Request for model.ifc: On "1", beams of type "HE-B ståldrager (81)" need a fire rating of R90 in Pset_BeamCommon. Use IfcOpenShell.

First a look at what the model holds.

```python
import ifcopenshell
import ifcopenshell.util.element

model = ifcopenshell.open("model.ifc")
print(model.schema)
storey = next(s for s in model.by_type("IfcBuildingStorey") if s.Name == "1")
beams = [e for e in ifcopenshell.util.element.get_decomposition(storey) if e.is_a("IfcBeam")]
seen = {}
for e in beams:
    element_type = ifcopenshell.util.element.get_type(e)
    key = (element_type.Name if element_type != e and element_type else None, ifcopenshell.util.element.get_pset(e, "Pset_BeamCommon", "FireRating"))
    seen[key] = seen.get(key, 0) + 1
for (name, value), count in sorted(seen.items(), key=str):
    print(count, "x", name, "|", value)
```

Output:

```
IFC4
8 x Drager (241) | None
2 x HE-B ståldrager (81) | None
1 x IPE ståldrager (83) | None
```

```python
import ifcopenshell
import ifcopenshell.api.pset
import ifcopenshell.util.element

model = ifcopenshell.open("model.ifc")

storey = next(s for s in model.by_type("IfcBuildingStorey") if s.Name == "1")
beams = [e for e in ifcopenshell.util.element.get_decomposition(storey) if e.is_a("IfcBeam")]

count = 0
for e in beams:
    element_type = ifcopenshell.util.element.get_type(e)
    if element_type in (None, e) or element_type.Name != "HE-B ståldrager (81)":
        continue
    # add_pset returns the element's existing set when there is one.
    pset = ifcopenshell.api.pset.add_pset(model, product=e, name="Pset_BeamCommon")
    ifcopenshell.api.pset.edit_pset(model, pset=pset, properties={"FireRating": "R90"})
    count += 1

print(count, "beams updated")

model.write("model_rev.ifc")
```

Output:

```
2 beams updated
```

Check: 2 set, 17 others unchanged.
